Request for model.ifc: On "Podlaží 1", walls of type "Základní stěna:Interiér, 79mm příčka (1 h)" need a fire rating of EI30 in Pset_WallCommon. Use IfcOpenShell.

First a look at what the model holds.

```python
import ifcopenshell
import ifcopenshell.util.element

model = ifcopenshell.open("model.ifc")
print(model.schema)
storey = next(s for s in model.by_type("IfcBuildingStorey") if s.Name == "Podlaží 1")
walls = [e for e in ifcopenshell.util.element.get_decomposition(storey) if e.is_a("IfcWall")]
seen = {}
for e in walls:
    element_type = ifcopenshell.util.element.get_type(e)
    key = (element_type.Name if element_type != e and element_type else None, ifcopenshell.util.element.get_pset(e, "Pset_WallCommon", "FireRating"))
    seen[key] = seen.get(key, 0) + 1
for (name, value), count in sorted(seen.items(), key=str):
    print(count, "x", name, "|", value)
```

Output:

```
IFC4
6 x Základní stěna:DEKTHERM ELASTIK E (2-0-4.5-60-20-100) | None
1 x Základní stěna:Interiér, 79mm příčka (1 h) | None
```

```python
import ifcopenshell
import ifcopenshell.api.pset
import ifcopenshell.util.element

model = ifcopenshell.open("model.ifc")

storey = next(s for s in model.by_type("IfcBuildingStorey") if s.Name == "Podlaží 1")
walls = [e for e in ifcopenshell.util.element.get_decomposition(storey) if e.is_a("IfcWall")]

count = 0
for e in walls:
    element_type = ifcopenshell.util.element.get_type(e)
    if element_type in (None, e) or element_type.Name != "Základní stěna:Interiér, 79mm příčka (1 h)":
        continue
    # add_pset returns the element's existing set when there is one.
    pset = ifcopenshell.api.pset.add_pset(model, product=e, name="Pset_WallCommon")
    ifcopenshell.api.pset.edit_pset(model, pset=pset, properties={"FireRating": "EI30"})
    count += 1

print(count, "walls updated")

model.write("model_edited.ifc")
```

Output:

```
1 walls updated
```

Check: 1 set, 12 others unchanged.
